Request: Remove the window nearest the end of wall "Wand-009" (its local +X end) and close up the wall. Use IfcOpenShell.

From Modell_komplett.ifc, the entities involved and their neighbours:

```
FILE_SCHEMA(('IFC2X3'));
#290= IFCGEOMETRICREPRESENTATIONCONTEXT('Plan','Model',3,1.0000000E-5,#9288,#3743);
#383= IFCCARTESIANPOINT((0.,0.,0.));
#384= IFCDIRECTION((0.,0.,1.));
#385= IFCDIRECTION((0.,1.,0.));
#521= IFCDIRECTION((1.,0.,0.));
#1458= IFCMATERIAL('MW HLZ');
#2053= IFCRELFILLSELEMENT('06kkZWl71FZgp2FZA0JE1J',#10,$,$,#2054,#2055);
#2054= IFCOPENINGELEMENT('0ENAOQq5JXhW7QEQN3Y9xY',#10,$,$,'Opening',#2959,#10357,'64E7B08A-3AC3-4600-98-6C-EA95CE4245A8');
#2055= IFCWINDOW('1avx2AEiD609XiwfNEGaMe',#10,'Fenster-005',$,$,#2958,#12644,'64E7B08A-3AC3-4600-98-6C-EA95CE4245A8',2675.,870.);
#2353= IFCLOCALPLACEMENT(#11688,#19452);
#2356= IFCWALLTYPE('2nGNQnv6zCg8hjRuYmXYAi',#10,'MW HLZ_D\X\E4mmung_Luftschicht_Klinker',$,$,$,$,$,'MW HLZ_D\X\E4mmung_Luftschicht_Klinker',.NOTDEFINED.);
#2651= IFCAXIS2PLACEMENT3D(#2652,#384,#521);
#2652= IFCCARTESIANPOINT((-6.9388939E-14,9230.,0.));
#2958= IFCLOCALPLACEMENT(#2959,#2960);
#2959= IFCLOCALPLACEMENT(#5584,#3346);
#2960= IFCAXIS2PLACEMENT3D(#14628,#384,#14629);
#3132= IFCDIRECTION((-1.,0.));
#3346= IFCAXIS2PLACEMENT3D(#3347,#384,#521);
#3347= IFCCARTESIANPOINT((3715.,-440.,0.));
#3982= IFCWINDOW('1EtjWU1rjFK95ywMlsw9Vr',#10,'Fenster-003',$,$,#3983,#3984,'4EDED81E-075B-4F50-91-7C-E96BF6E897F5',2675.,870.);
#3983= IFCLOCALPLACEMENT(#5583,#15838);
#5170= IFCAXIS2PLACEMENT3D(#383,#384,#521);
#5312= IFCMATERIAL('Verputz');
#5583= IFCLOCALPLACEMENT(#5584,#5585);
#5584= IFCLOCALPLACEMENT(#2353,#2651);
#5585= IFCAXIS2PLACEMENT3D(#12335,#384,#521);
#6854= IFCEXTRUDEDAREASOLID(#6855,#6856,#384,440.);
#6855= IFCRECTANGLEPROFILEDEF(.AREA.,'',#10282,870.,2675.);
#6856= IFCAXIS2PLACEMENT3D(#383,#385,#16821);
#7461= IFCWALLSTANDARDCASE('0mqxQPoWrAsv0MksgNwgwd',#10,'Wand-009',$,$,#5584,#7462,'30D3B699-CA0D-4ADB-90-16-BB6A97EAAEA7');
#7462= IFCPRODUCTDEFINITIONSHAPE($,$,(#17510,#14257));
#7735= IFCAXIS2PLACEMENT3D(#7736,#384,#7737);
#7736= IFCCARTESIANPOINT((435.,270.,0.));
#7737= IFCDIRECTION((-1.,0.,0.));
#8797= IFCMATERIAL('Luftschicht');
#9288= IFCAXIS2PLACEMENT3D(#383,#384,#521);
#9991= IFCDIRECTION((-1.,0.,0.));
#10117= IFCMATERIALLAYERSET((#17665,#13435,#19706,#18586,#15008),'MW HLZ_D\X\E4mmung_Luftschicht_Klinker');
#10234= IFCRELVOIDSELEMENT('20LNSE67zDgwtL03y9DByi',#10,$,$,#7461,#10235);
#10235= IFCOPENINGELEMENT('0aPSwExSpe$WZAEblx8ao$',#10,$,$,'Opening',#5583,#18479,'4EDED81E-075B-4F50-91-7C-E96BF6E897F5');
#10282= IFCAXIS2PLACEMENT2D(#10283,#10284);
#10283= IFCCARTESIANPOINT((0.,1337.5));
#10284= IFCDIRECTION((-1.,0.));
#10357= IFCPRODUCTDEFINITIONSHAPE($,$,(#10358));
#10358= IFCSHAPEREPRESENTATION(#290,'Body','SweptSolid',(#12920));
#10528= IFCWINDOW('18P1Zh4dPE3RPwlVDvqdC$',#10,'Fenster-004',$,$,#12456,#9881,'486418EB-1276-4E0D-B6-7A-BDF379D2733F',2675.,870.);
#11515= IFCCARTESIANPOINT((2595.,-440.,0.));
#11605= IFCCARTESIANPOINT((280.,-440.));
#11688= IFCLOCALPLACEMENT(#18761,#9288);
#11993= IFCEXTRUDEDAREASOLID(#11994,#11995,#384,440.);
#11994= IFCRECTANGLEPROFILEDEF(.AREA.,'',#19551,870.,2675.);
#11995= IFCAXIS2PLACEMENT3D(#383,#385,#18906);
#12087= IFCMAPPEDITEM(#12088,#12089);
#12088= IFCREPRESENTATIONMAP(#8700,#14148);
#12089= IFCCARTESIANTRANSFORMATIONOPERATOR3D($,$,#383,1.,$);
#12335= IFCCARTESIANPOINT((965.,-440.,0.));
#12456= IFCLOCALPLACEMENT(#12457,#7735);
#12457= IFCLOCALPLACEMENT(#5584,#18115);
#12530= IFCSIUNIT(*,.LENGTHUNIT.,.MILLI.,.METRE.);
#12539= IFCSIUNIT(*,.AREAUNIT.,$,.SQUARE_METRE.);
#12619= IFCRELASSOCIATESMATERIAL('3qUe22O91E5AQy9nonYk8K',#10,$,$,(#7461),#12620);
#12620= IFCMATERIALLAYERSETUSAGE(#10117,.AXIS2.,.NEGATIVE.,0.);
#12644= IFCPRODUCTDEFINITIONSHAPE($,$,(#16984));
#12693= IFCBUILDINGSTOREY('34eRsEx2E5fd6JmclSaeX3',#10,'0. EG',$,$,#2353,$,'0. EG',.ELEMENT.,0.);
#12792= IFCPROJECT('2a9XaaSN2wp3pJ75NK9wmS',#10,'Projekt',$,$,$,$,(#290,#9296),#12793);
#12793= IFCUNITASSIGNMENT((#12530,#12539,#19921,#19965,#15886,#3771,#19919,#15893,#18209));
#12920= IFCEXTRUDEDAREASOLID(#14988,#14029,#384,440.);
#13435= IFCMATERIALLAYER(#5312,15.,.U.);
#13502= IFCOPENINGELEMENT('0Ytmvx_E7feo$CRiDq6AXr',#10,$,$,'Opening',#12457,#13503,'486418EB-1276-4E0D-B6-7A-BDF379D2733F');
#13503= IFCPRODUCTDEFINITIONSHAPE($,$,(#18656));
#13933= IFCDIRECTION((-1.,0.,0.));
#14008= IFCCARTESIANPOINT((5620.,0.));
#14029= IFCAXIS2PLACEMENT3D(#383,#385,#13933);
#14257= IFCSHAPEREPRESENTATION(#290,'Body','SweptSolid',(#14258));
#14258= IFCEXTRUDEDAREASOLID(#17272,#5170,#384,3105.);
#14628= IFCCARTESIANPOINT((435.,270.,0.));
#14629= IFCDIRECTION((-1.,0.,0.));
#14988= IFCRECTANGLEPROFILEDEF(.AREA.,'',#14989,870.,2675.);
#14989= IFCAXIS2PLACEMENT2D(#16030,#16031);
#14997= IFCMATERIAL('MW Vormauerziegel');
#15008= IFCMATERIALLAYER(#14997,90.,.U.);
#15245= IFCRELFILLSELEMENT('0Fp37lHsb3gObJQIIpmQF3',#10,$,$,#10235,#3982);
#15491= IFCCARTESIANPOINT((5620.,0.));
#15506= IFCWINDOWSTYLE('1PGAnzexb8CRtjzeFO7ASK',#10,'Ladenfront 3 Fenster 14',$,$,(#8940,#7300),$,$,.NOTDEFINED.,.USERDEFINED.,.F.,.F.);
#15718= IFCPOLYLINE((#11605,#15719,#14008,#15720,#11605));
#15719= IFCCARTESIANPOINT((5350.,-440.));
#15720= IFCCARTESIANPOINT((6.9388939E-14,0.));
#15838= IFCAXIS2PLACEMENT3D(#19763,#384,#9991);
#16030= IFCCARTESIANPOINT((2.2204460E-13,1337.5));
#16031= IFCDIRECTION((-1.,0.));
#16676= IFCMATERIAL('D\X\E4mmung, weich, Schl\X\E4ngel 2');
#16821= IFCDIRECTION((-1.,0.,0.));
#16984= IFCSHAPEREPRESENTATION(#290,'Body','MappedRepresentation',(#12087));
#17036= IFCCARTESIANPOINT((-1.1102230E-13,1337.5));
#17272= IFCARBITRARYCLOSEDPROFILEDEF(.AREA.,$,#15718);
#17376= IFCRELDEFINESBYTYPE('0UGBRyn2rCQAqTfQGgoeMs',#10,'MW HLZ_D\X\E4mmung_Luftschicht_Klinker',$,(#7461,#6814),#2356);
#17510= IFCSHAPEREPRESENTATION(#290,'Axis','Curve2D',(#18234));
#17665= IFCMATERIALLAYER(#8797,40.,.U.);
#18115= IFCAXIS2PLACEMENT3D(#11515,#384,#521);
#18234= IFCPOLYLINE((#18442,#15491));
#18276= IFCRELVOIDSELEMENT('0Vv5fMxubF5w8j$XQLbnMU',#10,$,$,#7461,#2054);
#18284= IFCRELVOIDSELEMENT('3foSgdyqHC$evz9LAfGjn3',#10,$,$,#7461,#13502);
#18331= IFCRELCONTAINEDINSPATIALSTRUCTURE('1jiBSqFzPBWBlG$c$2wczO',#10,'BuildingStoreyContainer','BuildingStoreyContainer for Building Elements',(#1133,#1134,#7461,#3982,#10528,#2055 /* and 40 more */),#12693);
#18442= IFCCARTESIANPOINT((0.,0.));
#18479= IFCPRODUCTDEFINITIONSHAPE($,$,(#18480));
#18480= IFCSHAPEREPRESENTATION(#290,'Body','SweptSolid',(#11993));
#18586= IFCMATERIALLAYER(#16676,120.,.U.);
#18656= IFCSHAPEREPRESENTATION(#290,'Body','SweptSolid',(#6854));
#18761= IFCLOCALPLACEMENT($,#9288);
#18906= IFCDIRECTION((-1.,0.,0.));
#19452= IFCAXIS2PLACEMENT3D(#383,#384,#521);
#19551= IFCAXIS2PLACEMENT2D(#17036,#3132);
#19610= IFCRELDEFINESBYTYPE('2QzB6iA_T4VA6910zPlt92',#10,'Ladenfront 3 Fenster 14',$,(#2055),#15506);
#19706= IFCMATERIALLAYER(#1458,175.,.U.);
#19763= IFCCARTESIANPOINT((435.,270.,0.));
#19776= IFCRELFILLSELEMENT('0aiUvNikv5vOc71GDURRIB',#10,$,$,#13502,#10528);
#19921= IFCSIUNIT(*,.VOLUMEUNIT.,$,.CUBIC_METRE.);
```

```python
import ifcopenshell
import ifcopenshell.api.feature
import ifcopenshell.api.root
import ifcopenshell.geom
import ifcopenshell.util.shape

model = ifcopenshell.open("Modell_komplett.ifc")
settings = ifcopenshell.geom.settings()


def volume(element):
    """Net volume in cubic metres, openings subtracted."""
    shape = ifcopenshell.geom.create_shape(settings, element)
    return ifcopenshell.util.shape.get_volume(shape.geometry)


window = model.by_guid("1avx2AEiD609XiwfNEGaMe")
opening = window.FillsVoids[0].RelatingOpeningElement
wall = opening.VoidsElements[0].RelatingBuildingElement
before = volume(wall)

ifcopenshell.api.root.remove_product(model, product=window)
ifcopenshell.api.feature.remove_feature(model, feature=opening)

after = volume(wall)

print(f"wall volume {before:.3f} -> {after:.3f} m3")

model.write("Modell_komplett_v2.ifc")
```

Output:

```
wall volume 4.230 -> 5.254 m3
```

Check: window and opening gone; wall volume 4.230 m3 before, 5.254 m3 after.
